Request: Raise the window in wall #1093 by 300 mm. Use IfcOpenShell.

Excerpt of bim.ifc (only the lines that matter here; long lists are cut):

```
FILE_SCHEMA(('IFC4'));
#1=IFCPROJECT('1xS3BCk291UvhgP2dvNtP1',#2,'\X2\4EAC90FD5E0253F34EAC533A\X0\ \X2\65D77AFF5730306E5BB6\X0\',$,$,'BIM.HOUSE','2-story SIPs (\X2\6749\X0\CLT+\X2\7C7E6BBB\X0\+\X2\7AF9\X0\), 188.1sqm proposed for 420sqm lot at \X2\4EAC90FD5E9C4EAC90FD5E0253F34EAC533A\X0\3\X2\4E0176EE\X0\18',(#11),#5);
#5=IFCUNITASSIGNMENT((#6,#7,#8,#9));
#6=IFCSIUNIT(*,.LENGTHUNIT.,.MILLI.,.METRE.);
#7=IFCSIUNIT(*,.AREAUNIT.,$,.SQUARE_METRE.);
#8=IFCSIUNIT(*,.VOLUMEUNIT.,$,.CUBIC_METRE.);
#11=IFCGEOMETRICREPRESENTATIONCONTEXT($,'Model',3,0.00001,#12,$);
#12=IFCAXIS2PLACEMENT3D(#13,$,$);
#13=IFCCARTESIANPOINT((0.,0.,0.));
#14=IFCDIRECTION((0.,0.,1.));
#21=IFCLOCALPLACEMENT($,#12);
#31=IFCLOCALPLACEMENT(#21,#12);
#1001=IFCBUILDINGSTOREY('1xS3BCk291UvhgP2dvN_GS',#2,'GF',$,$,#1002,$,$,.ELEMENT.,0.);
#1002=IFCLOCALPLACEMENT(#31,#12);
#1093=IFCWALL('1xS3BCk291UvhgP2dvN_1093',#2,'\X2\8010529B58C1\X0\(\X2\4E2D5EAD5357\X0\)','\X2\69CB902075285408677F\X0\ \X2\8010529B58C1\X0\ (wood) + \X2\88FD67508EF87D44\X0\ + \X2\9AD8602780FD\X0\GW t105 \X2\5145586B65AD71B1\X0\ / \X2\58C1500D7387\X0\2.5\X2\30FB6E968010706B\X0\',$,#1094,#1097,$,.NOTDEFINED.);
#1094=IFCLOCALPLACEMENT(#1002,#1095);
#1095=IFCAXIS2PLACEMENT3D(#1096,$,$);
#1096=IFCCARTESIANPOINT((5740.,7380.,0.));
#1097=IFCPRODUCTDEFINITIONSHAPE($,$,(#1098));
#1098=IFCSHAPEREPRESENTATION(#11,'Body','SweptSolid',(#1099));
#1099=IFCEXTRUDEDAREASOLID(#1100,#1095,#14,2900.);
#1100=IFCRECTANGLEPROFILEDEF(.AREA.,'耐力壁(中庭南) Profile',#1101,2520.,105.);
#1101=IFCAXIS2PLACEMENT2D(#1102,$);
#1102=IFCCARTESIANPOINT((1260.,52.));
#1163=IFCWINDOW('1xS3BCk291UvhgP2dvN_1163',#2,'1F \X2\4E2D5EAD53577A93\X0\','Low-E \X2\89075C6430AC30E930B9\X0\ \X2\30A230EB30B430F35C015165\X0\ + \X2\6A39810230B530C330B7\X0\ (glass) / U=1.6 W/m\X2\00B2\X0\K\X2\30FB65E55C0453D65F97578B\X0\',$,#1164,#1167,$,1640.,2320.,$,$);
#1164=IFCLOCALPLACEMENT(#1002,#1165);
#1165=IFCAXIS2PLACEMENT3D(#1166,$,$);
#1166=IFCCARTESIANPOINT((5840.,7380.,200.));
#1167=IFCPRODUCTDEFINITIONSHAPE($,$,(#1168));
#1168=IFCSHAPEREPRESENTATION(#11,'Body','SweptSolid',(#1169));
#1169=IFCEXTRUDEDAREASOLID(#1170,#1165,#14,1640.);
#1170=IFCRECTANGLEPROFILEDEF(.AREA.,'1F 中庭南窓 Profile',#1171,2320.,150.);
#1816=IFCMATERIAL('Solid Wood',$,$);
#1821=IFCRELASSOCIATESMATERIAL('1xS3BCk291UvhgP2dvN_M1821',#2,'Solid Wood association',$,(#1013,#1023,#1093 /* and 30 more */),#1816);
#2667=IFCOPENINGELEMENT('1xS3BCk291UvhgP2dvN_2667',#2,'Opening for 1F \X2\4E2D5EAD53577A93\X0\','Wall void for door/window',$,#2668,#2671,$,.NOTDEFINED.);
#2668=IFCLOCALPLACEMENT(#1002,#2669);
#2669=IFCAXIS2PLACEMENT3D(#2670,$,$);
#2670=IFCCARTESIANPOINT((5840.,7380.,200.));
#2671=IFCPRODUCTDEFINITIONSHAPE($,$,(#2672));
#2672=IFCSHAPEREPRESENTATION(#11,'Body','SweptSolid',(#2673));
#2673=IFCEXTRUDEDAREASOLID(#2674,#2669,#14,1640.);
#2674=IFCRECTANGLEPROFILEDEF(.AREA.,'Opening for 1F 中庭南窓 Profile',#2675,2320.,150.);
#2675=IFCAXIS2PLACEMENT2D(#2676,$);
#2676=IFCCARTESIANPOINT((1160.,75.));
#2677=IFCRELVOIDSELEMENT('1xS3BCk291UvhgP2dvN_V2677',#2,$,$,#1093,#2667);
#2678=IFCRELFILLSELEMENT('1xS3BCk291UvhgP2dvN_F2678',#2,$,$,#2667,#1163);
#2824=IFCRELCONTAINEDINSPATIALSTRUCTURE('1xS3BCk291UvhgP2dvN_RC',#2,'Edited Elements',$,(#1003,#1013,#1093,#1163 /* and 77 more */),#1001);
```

```python
import numpy as np
import ifcopenshell
import ifcopenshell.api.geometry
import ifcopenshell.util.placement
import ifcopenshell.util.unit

model = ifcopenshell.open("bim.ifc")
unit_scale = ifcopenshell.util.unit.calculate_unit_scale(model)

window = model.by_id(1163)
opening = window.FillsVoids[0].RelatingOpeningElement
dz = 0.3 / unit_scale

shift = np.array([0.0, 0.0, dz])
# The window is not placed relative to its opening, so move both.
for product in (opening, window):
    matrix = ifcopenshell.util.placement.get_local_placement(product.ObjectPlacement)
    matrix[:3, 3] += shift
    ifcopenshell.api.geometry.edit_object_placement(model, product=product, matrix=matrix, is_si=False)

print(f"moved by {dz * unit_scale:+.3f} m")

model.write("bim-out.ifc")
```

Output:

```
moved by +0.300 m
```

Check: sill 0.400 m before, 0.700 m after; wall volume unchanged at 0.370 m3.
